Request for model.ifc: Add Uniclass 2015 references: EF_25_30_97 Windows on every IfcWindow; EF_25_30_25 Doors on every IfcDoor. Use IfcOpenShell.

First a look at what the model holds.

```python
import ifcopenshell

model = ifcopenshell.open("model.ifc")
print(model.schema)
print("classifications:", [c.Name for c in model.by_type("IfcClassification")])
for ifc_class in ("IfcDoor", "IfcRoof", "IfcStair", "IfcWall", "IfcWindow"):
    print(ifc_class, len(model.by_type(ifc_class)))
```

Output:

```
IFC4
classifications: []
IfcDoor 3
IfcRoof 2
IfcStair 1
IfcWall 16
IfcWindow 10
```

```python
import ifcopenshell
import ifcopenshell.api.classification

model = ifcopenshell.open("model.ifc")

system = ifcopenshell.api.classification.add_classification(model, classification="Uniclass 2015")

codes = {
    "IfcWindow": ("EF_25_30_97", "Windows"),
    "IfcDoor": ("EF_25_30_25", "Doors"),
}
for ifc_class, (code, name) in codes.items():
    products = model.by_type(ifc_class)
    ifcopenshell.api.classification.add_reference(
        model, products=products, classification=system, identification=code, name=name
    )
    print(code, len(products))

model.write("model_rev.ifc")
```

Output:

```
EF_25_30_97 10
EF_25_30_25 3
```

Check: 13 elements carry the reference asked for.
